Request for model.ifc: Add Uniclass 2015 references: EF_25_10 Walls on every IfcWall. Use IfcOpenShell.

First a look at what the model holds.

```python
import ifcopenshell

model = ifcopenshell.open("model.ifc")
print(model.schema)
print("classifications:", [c.Name for c in model.by_type("IfcClassification")])
for ifc_class in ("IfcDoor", "IfcRoof", "IfcStair", "IfcWall", "IfcWindow"):
    print(ifc_class, len(model.by_type(ifc_class)))
```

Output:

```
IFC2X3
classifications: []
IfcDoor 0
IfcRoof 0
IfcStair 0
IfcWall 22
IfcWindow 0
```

```python
import ifcopenshell
import ifcopenshell.api.classification

model = ifcopenshell.open("model.ifc")

# IFC2X3 requires Source and Edition and has no link from the project to the system.
system = model.create_entity("IfcClassification", Source="NBS", Edition="2015", Name="Uniclass 2015")

codes = {
    "IfcWall": ("EF_25_10", "Walls"),
}
for ifc_class, (code, name) in codes.items():
    products = model.by_type(ifc_class)
    ifcopenshell.api.classification.add_reference(
        model, products=products, classification=system, identification=code, name=name
    )
    print(code, len(products))

model.write("model_updated.ifc")
```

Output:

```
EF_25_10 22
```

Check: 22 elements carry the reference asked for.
